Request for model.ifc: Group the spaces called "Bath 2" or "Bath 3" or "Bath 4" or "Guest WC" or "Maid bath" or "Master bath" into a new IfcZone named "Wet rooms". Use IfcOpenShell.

First a look at what the model holds.

```python
import ifcopenshell

model = ifcopenshell.open("model.ifc")
print(model.schema)
seen = {}
for space in model.by_type("IfcSpace"):
    seen[space.LongName] = seen.get(space.LongName, 0) + 1
for name, count in sorted(seen.items(), key=str):
    print(count, "x", name)
print("zones:", [z.Name for z in model.by_type("IfcZone")][:20])
```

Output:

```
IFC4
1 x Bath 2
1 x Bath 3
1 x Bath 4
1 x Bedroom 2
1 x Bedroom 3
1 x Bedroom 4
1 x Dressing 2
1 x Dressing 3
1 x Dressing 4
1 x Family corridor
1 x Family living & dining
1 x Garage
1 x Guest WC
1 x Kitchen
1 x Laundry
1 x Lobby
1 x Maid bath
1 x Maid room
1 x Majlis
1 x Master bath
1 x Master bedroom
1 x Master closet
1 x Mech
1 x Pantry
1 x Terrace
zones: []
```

```python
import ifcopenshell
import ifcopenshell.api.group
import ifcopenshell.api.root

model = ifcopenshell.open("model.ifc")

names = {"Bath 2", "Bath 3", "Bath 4", "Guest WC", "Maid bath", "Master bath"}
spaces = [s for s in model.by_type("IfcSpace") if s.LongName in names]

zone = ifcopenshell.api.root.create_entity(model, ifc_class="IfcZone", name="Wet rooms")
ifcopenshell.api.group.assign_group(model, products=spaces, group=zone)
print(len(spaces), "spaces in", zone.Name)

model.write("model_v2.ifc")
```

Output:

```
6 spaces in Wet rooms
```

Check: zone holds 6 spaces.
